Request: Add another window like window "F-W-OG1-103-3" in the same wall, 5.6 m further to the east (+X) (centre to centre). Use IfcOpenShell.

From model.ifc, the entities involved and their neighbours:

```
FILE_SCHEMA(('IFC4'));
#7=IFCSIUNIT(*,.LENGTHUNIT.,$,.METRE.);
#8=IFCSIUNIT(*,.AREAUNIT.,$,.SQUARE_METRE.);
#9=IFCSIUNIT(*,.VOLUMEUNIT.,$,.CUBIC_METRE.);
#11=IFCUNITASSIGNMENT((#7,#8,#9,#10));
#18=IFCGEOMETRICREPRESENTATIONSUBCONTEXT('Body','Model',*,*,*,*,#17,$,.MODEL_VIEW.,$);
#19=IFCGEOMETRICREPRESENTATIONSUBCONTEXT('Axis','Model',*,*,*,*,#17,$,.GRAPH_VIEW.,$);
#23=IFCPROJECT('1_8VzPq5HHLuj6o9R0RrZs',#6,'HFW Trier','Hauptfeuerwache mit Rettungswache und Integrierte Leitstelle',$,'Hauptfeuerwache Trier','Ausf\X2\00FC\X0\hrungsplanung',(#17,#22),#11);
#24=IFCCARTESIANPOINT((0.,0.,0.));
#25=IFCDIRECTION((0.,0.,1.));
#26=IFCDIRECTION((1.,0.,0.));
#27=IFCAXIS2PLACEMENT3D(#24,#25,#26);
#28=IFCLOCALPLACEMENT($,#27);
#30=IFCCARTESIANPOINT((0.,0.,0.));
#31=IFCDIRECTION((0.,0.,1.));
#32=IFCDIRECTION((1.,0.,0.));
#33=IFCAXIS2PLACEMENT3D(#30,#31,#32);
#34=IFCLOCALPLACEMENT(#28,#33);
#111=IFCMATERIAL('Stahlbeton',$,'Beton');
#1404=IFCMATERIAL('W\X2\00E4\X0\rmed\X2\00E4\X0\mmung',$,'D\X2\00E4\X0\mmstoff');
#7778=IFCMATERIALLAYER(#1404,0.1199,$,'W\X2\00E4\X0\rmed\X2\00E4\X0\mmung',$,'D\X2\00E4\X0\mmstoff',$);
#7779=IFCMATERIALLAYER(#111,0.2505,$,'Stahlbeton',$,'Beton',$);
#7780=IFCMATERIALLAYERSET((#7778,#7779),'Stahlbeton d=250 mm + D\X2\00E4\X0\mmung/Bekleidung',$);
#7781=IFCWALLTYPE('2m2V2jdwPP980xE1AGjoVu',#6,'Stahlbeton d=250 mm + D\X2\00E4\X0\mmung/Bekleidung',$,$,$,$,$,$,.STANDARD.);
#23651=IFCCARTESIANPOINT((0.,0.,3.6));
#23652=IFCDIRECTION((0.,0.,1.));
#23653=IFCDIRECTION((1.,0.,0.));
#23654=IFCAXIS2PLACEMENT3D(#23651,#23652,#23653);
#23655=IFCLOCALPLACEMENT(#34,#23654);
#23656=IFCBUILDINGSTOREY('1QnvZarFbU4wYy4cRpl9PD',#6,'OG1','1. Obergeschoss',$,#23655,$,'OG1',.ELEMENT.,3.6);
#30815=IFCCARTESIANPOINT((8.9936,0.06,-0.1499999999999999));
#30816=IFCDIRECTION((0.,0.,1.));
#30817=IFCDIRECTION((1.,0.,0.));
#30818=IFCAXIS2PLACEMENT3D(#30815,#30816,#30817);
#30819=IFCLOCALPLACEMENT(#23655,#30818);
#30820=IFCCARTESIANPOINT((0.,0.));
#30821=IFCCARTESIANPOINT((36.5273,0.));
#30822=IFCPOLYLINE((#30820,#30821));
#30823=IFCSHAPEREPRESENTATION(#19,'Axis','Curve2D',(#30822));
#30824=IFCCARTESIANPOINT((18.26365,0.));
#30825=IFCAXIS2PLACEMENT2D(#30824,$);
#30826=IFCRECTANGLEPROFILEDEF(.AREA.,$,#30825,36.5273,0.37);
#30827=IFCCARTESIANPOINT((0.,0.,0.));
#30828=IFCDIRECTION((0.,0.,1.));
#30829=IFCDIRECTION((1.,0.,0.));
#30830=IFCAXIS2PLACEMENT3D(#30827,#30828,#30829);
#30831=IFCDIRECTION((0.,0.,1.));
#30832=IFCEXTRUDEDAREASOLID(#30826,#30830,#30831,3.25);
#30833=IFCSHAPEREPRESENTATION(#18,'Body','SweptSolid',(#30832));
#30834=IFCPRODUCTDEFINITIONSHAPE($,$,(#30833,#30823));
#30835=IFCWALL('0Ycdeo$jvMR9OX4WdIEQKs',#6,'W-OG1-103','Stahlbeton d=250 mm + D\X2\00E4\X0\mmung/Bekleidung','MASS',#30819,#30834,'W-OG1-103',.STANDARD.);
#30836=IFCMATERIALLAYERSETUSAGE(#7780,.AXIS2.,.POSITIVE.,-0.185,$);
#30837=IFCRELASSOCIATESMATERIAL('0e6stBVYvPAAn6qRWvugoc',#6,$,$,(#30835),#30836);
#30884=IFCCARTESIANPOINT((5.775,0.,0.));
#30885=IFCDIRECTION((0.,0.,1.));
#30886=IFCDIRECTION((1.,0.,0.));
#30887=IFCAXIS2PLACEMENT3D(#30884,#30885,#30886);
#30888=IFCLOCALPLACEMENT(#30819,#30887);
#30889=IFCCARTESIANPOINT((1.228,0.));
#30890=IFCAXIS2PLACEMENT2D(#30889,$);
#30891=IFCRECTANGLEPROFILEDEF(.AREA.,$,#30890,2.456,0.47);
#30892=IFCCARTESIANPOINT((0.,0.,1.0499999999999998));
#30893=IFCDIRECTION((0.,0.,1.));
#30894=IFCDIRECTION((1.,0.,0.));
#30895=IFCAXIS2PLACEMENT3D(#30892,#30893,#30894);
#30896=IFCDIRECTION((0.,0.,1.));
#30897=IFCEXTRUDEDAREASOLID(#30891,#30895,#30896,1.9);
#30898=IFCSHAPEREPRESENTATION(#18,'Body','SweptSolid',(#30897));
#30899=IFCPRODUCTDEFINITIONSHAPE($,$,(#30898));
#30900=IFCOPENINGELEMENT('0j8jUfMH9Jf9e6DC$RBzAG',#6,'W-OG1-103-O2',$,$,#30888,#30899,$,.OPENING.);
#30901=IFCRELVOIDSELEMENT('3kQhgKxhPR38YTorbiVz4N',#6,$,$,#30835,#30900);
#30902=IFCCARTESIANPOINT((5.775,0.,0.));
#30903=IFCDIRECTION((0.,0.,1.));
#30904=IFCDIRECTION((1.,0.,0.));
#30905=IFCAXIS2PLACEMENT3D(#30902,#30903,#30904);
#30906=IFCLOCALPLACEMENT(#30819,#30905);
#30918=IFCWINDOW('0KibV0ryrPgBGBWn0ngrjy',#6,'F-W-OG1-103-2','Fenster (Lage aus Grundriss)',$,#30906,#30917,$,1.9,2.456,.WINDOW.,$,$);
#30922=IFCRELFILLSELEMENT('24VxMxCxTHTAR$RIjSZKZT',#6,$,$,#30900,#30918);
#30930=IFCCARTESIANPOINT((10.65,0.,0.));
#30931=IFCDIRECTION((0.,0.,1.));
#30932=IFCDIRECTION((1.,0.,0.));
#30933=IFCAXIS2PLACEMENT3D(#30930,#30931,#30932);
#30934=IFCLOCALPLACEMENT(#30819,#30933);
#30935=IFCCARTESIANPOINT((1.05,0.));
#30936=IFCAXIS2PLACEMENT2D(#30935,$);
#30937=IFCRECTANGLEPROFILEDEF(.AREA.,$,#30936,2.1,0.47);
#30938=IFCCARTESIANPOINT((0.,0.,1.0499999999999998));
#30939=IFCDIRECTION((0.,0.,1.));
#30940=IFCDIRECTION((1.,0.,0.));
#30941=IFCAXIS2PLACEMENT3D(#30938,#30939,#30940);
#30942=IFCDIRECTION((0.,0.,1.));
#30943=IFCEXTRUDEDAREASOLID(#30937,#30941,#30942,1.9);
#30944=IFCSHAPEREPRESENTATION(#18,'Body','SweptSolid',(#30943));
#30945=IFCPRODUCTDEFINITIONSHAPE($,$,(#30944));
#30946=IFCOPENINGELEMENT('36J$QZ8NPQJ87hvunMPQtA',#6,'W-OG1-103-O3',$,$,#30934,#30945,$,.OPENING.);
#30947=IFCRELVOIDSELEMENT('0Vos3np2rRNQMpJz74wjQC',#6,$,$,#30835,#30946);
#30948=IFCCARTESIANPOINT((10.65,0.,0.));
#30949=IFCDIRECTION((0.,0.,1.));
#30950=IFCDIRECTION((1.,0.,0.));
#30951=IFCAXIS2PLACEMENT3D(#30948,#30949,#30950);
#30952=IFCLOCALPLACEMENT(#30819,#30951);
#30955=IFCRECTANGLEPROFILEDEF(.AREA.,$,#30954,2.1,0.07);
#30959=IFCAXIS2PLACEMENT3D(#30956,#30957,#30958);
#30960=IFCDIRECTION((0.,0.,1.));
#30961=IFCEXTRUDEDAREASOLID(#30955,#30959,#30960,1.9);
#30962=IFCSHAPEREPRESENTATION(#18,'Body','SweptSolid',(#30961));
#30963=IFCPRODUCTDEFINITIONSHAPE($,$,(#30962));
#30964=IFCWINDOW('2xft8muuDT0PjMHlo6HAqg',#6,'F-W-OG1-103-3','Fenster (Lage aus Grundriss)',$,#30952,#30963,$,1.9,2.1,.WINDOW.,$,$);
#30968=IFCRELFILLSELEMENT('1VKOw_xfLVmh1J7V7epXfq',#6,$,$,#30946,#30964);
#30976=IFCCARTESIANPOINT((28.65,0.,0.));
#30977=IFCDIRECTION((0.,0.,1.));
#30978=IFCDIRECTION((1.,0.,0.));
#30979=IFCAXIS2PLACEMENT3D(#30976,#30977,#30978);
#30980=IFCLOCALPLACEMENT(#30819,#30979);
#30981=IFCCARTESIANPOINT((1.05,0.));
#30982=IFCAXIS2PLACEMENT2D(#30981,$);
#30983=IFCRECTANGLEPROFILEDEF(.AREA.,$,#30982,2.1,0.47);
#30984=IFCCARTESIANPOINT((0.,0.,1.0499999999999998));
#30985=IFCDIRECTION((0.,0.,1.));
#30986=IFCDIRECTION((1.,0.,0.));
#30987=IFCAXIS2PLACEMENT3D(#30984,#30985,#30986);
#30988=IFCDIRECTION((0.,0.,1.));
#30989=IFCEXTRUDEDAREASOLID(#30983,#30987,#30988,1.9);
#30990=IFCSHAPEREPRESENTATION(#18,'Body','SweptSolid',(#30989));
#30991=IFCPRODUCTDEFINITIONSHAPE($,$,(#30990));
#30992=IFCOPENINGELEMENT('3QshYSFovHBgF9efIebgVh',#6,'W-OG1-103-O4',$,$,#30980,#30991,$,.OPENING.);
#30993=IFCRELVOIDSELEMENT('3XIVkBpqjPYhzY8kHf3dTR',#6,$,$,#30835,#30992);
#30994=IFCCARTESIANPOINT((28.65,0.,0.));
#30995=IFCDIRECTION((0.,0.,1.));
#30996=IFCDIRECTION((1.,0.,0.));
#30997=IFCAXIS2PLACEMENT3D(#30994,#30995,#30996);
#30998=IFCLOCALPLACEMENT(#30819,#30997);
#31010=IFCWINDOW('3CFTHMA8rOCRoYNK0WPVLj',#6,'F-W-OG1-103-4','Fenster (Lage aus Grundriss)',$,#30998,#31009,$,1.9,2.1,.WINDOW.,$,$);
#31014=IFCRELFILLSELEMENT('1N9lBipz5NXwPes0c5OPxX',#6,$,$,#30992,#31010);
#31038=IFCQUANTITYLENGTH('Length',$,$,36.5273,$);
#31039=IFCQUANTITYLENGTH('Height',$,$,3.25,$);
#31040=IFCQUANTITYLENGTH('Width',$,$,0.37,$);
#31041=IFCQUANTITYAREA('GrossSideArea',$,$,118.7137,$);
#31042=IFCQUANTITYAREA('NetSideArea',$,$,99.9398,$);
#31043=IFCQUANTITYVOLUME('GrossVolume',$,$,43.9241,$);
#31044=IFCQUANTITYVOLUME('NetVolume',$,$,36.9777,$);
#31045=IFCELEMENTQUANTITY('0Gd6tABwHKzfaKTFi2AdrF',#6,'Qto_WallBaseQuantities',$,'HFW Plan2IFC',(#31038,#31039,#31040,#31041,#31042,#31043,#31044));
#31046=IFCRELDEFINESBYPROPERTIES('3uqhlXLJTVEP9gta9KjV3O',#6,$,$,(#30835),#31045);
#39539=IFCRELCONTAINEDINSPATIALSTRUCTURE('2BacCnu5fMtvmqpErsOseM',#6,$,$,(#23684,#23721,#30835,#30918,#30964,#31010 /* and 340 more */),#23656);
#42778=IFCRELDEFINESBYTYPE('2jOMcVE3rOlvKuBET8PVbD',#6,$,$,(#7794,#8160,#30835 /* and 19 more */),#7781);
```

```python
import ifcopenshell
import ifcopenshell.api.feature
import ifcopenshell.api.geometry
import ifcopenshell.api.pset
import ifcopenshell.api.root
import ifcopenshell.geom
import ifcopenshell.util.element
import ifcopenshell.util.placement
import ifcopenshell.util.shape
import ifcopenshell.util.unit

model = ifcopenshell.open("model.ifc")
unit_scale = ifcopenshell.util.unit.calculate_unit_scale(model)
area_scale = ifcopenshell.util.unit.calculate_unit_scale(model, "AREAUNIT")
volume_scale = ifcopenshell.util.unit.calculate_unit_scale(model, "VOLUMEUNIT")
settings = ifcopenshell.geom.settings()


def volume(element):
    """Net volume in cubic metres, openings subtracted."""
    shape = ifcopenshell.geom.create_shape(settings, element)
    return ifcopenshell.util.shape.get_volume(shape.geometry)


def reuse_history(source, copy):
    """copy_class also copies each property set's owner history, people and application; keep the originals."""
    for rel in copy.IsDefinedBy:
        if rel.is_a("IfcRelDefinesByProperties") and (history := rel.RelatingPropertyDefinition.OwnerHistory):
            rel.RelatingPropertyDefinition.OwnerHistory = source.OwnerHistory
            ifcopenshell.util.element.remove_deep2(model, history)


window = model.by_guid("2xft8muuDT0PjMHlo6HAqg")
opening = window.FillsVoids[0].RelatingOpeningElement
wall = opening.VoidsElements[0].RelatingBuildingElement
before = volume(wall)
shift = ifcopenshell.util.placement.get_local_placement(wall.ObjectPlacement)[:3, 0] * 5.6 / unit_scale

# copy_class copies the void relationship, type, container and properties, but no geometry.
new_opening = ifcopenshell.api.root.copy_class(model, product=opening)
new_opening.Representation = ifcopenshell.util.element.copy_deep(
    model, opening.Representation, exclude=["IfcGeometricRepresentationContext", "IfcRepresentationMap"]
)
new_window = ifcopenshell.api.root.copy_class(model, product=window)
new_window.Representation = ifcopenshell.util.element.copy_deep(
    model, window.Representation, exclude=["IfcGeometricRepresentationContext", "IfcRepresentationMap"]
)
reuse_history(window, new_window)
ifcopenshell.api.feature.add_filling(model, opening=new_opening, element=new_window)

for old, new in ((opening, new_opening), (window, new_window)):
    matrix = ifcopenshell.util.placement.get_local_placement(old.ObjectPlacement)
    matrix[:3, 3] += shift
    ifcopenshell.api.geometry.edit_object_placement(model, product=new, matrix=matrix, is_si=False)

after = volume(wall)
thickness = 0.37  # wall thickness in metres

# Update the wall's stored quantities.
qto = model.by_id(ifcopenshell.util.element.get_pset(wall, "Qto_WallBaseQuantities", should_inherit=False)["id"])
ifcopenshell.api.pset.edit_qto(model, qto=qto, properties={
    "NetSideArea": after / thickness / area_scale,
    "NetVolume": after / volume_scale,
})

print(f"wall volume {before:.3f} -> {after:.3f} m3")

model.write("model_rev.ifc")
```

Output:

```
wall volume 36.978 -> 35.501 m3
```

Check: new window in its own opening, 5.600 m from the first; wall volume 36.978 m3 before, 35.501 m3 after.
